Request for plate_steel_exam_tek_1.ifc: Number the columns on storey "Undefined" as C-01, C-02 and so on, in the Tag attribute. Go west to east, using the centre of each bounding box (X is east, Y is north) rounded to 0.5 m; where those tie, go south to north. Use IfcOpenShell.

First a look at what the model holds.

```python
import ifcopenshell
import ifcopenshell.util.element
import ifcopenshell.util.placement

model = ifcopenshell.open("plate_steel_exam_tek_1.ifc")
print(model.schema)
storey = next(s for s in model.by_type("IfcBuildingStorey") if s.Name == "Undefined")
columns = [e for e in ifcopenshell.util.element.get_decomposition(storey) if e.is_a("IfcColumn")]
for e in sorted(columns, key=lambda e: e.id()):
    origin = ifcopenshell.util.placement.get_local_placement(e.ObjectPlacement)[:3, 3]
    print(e.id(), e.Tag, e.Name, origin.round(2) + 0.0, sep=" | ")
```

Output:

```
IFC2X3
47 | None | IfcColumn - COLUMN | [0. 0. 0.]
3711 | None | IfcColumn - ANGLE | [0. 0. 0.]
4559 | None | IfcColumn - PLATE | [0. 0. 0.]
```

```python
import ifcopenshell
import ifcopenshell.geom
import ifcopenshell.util.element
import ifcopenshell.util.shape

model = ifcopenshell.open("plate_steel_exam_tek_1.ifc")
settings = ifcopenshell.geom.settings()
settings.set("use-world-coords", True)


def centre(element):
    shape = ifcopenshell.geom.create_shape(settings, element)
    return ifcopenshell.util.shape.get_bbox_centroid(shape.geometry)


storey = next(s for s in model.by_type("IfcBuildingStorey") if s.Name == "Undefined")
columns = [e for e in ifcopenshell.util.element.get_decomposition(storey) if e.is_a("IfcColumn")]

# Insertion points can sit at a corner or the storey origin, so sort by the geometry (in metres).
centres = {e: centre(e) for e in columns}
columns.sort(key=lambda e: (round(centres[e][0] / 0.5), centres[e][1]))

for i, e in enumerate(columns, start=1):
    number = f"C-{i:02d}"
    e.Tag = number
    print(e.id(), number)

model.write("plate_steel_exam_tek_1_rev.ifc")
```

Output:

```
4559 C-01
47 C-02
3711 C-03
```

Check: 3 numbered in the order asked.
